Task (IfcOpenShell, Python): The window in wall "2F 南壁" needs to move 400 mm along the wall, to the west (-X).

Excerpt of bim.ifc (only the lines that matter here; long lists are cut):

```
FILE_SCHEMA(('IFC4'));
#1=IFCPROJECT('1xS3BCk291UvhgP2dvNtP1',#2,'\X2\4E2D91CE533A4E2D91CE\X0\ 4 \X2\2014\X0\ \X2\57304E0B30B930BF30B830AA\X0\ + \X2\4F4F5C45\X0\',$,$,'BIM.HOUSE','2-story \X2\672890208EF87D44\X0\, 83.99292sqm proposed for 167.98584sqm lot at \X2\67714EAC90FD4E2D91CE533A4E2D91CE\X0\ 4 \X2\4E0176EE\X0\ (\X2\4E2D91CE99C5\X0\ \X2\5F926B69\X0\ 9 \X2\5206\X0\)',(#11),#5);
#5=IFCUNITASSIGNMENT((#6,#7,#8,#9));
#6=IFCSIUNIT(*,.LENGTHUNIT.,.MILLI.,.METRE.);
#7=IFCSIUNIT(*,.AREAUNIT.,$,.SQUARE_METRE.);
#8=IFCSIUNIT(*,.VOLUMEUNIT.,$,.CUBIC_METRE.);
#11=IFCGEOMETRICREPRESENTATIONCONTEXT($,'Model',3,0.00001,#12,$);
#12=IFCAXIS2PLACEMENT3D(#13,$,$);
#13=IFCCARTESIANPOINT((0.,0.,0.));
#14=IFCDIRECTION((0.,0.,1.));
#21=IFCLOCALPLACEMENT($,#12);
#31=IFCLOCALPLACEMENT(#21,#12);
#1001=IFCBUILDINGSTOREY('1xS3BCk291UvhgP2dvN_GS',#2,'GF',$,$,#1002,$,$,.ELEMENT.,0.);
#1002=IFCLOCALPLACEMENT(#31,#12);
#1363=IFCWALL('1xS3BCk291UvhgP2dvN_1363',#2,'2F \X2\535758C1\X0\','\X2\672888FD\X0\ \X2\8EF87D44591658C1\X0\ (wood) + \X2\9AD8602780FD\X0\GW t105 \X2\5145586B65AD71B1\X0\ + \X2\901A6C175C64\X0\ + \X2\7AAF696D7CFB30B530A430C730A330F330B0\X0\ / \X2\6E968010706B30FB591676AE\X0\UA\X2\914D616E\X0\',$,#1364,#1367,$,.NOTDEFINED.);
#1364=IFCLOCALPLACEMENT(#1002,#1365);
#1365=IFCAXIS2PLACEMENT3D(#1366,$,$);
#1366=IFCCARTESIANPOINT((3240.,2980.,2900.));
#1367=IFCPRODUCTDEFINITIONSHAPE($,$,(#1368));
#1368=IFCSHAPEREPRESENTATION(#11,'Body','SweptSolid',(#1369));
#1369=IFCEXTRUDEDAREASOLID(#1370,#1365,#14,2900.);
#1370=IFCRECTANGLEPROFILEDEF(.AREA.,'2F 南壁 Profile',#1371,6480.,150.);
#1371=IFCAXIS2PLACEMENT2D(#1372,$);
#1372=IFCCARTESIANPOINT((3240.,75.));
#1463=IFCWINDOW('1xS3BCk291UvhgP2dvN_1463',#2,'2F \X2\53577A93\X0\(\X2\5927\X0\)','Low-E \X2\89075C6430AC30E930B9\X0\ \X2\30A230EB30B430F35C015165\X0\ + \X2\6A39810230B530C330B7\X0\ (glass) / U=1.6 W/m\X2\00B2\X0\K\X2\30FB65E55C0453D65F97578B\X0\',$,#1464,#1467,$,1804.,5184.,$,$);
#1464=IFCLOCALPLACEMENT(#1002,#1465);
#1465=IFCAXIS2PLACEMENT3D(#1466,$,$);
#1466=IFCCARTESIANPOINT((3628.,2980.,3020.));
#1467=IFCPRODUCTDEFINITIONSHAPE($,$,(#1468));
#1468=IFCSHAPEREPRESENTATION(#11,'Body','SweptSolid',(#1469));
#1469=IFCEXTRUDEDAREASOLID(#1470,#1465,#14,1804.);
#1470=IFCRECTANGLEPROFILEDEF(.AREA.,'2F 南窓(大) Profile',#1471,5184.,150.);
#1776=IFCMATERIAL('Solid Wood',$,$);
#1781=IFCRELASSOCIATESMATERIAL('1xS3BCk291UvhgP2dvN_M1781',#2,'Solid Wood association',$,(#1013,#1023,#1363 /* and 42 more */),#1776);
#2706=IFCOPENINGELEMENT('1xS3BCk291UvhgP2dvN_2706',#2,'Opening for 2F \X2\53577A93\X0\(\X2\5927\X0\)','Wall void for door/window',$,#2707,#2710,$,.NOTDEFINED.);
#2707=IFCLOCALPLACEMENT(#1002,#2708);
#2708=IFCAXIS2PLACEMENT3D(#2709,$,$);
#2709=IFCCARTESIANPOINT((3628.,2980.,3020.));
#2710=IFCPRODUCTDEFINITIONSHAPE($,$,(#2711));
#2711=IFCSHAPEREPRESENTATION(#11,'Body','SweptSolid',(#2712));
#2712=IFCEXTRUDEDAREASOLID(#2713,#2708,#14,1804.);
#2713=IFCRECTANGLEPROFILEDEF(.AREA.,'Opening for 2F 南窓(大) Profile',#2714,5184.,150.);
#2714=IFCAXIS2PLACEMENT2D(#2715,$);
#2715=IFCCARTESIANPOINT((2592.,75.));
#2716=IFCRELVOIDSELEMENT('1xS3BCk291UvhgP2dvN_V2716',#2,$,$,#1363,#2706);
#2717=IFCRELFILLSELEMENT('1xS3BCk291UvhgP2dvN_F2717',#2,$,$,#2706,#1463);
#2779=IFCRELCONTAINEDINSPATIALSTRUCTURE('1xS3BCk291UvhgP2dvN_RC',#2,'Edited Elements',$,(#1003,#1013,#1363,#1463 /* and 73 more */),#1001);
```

```python
import ifcopenshell
import ifcopenshell.api.geometry
import ifcopenshell.util.placement
import ifcopenshell.util.unit

model = ifcopenshell.open("bim.ifc")
unit_scale = ifcopenshell.util.unit.calculate_unit_scale(model)

window = model.by_id(1463)
opening = window.FillsVoids[0].RelatingOpeningElement
wall = opening.VoidsElements[0].RelatingBuildingElement

wall_matrix = ifcopenshell.util.placement.get_local_placement(wall.ObjectPlacement)
shift = wall_matrix[:3, 0] * -0.4 / unit_scale
before = ifcopenshell.util.placement.get_local_placement(window.ObjectPlacement)[:3, 3].copy()

# The window is not placed relative to its opening, so move both.
for product in (opening, window):
    matrix = ifcopenshell.util.placement.get_local_placement(product.ObjectPlacement)
    matrix[:3, 3] += shift
    ifcopenshell.api.geometry.edit_object_placement(model, product=product, matrix=matrix, is_si=False)

after = ifcopenshell.util.placement.get_local_placement(window.ObjectPlacement)[:3, 3]
print("window moved by", (after - before).round(3) + 0.0)

model.write("bim_edited.ifc")
```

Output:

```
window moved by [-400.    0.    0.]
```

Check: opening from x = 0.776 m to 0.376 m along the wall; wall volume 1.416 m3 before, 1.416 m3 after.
